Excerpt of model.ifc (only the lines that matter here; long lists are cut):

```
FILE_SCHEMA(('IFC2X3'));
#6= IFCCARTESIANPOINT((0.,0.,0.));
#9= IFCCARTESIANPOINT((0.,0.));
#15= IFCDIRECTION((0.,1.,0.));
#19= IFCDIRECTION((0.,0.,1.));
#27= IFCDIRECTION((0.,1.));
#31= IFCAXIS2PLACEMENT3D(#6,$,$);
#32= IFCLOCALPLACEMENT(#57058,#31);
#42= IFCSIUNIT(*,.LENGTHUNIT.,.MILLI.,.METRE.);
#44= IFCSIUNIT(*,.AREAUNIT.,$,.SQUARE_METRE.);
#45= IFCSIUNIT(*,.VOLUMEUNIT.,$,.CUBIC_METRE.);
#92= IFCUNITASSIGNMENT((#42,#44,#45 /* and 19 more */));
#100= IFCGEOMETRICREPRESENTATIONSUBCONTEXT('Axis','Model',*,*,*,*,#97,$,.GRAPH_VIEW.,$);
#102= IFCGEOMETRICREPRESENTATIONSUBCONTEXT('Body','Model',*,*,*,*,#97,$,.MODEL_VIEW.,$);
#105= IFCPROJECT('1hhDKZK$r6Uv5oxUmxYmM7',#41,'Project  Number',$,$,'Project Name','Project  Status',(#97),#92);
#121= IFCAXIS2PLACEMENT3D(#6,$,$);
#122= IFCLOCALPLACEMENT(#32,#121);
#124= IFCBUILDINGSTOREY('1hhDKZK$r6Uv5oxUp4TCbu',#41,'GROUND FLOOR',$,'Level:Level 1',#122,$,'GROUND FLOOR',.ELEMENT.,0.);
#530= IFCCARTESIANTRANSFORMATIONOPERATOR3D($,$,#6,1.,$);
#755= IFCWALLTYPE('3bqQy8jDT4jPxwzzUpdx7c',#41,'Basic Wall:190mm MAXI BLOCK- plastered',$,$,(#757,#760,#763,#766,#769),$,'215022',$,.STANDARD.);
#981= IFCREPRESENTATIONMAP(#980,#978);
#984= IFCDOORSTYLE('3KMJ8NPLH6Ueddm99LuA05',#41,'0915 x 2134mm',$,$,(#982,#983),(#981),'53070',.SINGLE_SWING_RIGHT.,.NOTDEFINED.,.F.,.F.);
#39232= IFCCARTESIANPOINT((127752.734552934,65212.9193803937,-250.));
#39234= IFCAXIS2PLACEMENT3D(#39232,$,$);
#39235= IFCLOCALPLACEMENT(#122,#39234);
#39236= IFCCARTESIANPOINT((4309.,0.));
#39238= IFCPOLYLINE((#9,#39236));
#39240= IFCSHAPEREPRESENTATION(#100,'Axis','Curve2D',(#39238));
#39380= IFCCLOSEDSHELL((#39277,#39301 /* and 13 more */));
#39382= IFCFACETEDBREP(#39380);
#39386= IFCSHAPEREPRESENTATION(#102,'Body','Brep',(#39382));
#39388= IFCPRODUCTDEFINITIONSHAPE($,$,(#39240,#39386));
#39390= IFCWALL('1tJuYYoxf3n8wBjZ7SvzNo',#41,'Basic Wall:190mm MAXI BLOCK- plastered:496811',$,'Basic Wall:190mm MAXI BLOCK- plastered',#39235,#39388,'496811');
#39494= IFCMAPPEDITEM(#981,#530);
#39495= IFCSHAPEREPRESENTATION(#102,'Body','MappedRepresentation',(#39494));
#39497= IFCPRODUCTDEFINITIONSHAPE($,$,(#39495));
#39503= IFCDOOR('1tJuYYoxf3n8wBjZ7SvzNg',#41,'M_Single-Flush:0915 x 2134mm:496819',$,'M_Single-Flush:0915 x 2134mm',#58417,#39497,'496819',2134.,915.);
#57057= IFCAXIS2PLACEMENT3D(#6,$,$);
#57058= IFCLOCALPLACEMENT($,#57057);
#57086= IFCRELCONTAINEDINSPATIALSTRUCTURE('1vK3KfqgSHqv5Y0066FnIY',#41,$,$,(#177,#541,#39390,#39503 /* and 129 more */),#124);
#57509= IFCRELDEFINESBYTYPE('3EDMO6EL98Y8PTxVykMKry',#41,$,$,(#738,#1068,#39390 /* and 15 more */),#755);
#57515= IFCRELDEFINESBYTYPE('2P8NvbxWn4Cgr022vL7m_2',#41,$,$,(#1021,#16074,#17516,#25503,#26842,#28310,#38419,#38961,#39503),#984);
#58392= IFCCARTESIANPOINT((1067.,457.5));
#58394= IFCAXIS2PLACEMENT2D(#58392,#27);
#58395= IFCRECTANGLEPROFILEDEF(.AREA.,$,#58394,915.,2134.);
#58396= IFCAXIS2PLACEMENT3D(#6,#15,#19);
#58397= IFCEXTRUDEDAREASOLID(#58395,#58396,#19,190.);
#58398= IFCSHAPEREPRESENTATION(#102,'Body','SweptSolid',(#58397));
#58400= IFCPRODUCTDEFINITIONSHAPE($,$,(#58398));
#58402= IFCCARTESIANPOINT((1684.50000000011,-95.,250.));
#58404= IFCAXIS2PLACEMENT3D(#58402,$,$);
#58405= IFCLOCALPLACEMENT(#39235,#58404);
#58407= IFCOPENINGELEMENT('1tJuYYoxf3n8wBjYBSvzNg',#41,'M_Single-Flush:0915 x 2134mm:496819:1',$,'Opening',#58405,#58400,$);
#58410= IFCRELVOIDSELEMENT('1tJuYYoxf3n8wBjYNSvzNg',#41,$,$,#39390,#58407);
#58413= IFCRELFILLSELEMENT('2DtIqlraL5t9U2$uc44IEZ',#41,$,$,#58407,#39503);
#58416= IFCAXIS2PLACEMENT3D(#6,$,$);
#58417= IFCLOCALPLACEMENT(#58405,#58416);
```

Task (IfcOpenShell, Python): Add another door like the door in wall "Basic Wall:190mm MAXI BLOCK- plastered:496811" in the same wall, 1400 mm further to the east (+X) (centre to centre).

```python
import ifcopenshell
import ifcopenshell.api.feature
import ifcopenshell.api.geometry
import ifcopenshell.api.root
import ifcopenshell.geom
import ifcopenshell.util.element
import ifcopenshell.util.placement
import ifcopenshell.util.shape

model = ifcopenshell.open("model.ifc")
settings = ifcopenshell.geom.settings()


def volume(element):
    """Net volume in cubic metres, openings subtracted."""
    shape = ifcopenshell.geom.create_shape(settings, element)
    return ifcopenshell.util.shape.get_volume(shape.geometry)


def reuse_history(source, copy):
    """copy_class also copies each property set's owner history, people and application; keep the originals."""
    for rel in copy.IsDefinedBy:
        if rel.is_a("IfcRelDefinesByProperties") and (history := rel.RelatingPropertyDefinition.OwnerHistory):
            rel.RelatingPropertyDefinition.OwnerHistory = source.OwnerHistory
            ifcopenshell.util.element.remove_deep2(model, history)


door = model.by_guid("1tJuYYoxf3n8wBjZ7SvzNg")
opening = door.FillsVoids[0].RelatingOpeningElement
wall = opening.VoidsElements[0].RelatingBuildingElement
before = volume(wall)
shift = ifcopenshell.util.placement.get_local_placement(wall.ObjectPlacement)[:3, 0] * 1400.0

# copy_class copies the void relationship, type, container and properties, but no geometry.
new_opening = ifcopenshell.api.root.copy_class(model, product=opening)
new_opening.Representation = ifcopenshell.util.element.copy_deep(
    model, opening.Representation, exclude=["IfcGeometricRepresentationContext", "IfcRepresentationMap"]
)
new_opening.Name = "M_Single-Flush:0915 x 2134mm"
new_door = ifcopenshell.api.root.copy_class(model, product=door)
new_door.Representation = ifcopenshell.util.element.copy_deep(
    model, door.Representation, exclude=["IfcGeometricRepresentationContext", "IfcRepresentationMap"]
)
new_door.Name = "M_Single-Flush:0915 x 2134mm"
new_door.Tag = None
reuse_history(door, new_door)
fills = ifcopenshell.api.feature.add_filling(model, opening=new_opening, element=new_door)
fills.OwnerHistory = new_door.OwnerHistory  # required in IFC2X3

for old, new in ((opening, new_opening), (door, new_door)):
    matrix = ifcopenshell.util.placement.get_local_placement(old.ObjectPlacement)
    matrix[:3, 3] += shift
    ifcopenshell.api.geometry.edit_object_placement(model, product=new, matrix=matrix, is_si=False)

after = volume(wall)

print(f"wall volume {before:.3f} -> {after:.3f} m3")

model.write("model_v2.ifc")
```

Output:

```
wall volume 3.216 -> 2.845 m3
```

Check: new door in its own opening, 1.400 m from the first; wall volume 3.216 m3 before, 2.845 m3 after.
